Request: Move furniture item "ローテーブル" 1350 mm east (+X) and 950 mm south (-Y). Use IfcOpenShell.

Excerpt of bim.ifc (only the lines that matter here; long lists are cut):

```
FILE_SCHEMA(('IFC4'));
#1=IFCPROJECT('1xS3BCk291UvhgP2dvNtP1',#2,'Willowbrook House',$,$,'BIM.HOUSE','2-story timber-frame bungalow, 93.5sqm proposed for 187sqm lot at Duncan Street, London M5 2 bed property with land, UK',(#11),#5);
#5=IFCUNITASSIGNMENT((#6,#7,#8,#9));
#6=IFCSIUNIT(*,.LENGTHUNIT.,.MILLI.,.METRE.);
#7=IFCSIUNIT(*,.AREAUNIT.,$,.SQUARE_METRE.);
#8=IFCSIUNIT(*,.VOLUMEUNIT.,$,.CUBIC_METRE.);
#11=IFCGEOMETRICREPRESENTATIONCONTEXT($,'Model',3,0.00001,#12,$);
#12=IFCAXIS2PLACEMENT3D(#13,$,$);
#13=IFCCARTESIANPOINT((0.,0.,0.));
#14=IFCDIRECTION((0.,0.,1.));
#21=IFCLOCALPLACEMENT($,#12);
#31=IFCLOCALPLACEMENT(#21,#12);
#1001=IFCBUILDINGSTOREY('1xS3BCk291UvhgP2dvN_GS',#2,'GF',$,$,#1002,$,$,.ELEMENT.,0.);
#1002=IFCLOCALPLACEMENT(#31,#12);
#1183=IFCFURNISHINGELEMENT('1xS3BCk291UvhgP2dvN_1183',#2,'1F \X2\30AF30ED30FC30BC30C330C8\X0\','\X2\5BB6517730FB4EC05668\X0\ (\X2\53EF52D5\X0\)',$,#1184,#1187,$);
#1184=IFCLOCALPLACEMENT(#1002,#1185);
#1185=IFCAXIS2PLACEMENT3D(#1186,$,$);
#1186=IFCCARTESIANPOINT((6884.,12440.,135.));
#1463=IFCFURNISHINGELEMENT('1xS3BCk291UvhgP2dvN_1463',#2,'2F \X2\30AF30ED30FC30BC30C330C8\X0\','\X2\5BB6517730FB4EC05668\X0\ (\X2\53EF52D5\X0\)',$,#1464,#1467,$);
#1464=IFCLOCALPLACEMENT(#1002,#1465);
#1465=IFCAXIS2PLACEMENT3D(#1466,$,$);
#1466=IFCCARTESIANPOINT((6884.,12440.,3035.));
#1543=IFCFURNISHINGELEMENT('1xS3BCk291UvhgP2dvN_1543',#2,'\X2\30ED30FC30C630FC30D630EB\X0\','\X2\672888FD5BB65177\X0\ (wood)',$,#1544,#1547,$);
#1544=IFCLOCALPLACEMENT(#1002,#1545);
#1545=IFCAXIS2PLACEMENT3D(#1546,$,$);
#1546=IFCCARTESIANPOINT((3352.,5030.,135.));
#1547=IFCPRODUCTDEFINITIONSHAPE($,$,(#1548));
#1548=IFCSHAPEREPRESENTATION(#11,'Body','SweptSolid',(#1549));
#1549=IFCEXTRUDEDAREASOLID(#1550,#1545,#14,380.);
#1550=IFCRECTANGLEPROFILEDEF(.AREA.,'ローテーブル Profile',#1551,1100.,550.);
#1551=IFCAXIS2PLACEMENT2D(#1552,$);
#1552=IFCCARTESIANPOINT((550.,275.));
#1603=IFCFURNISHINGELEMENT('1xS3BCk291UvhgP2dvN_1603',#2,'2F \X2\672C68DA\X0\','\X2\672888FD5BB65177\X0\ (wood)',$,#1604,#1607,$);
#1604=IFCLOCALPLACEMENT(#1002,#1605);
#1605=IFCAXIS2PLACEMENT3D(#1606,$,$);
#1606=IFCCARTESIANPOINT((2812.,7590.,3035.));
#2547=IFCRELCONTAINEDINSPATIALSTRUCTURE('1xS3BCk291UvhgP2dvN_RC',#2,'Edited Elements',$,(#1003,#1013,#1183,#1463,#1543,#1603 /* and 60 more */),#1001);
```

```python
import ifcopenshell
import ifcopenshell.api.geometry
import ifcopenshell.util.placement
import ifcopenshell.util.unit

model = ifcopenshell.open("bim.ifc")
unit_scale = ifcopenshell.util.unit.calculate_unit_scale(model)

item = model.by_id(1543)
matrix = ifcopenshell.util.placement.get_local_placement(item.ObjectPlacement)
matrix[0, 3] += 1.35 / unit_scale
matrix[1, 3] -= 0.95 / unit_scale
ifcopenshell.api.geometry.edit_object_placement(model, product=item, matrix=matrix, is_si=False)

print(ifcopenshell.util.placement.get_local_placement(item.ObjectPlacement).round(3) + 0.0)

model.write("bim_updated.ifc")
```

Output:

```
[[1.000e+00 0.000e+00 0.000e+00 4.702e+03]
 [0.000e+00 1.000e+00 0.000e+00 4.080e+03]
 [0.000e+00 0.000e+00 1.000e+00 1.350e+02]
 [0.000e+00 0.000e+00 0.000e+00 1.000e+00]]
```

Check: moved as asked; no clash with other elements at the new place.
